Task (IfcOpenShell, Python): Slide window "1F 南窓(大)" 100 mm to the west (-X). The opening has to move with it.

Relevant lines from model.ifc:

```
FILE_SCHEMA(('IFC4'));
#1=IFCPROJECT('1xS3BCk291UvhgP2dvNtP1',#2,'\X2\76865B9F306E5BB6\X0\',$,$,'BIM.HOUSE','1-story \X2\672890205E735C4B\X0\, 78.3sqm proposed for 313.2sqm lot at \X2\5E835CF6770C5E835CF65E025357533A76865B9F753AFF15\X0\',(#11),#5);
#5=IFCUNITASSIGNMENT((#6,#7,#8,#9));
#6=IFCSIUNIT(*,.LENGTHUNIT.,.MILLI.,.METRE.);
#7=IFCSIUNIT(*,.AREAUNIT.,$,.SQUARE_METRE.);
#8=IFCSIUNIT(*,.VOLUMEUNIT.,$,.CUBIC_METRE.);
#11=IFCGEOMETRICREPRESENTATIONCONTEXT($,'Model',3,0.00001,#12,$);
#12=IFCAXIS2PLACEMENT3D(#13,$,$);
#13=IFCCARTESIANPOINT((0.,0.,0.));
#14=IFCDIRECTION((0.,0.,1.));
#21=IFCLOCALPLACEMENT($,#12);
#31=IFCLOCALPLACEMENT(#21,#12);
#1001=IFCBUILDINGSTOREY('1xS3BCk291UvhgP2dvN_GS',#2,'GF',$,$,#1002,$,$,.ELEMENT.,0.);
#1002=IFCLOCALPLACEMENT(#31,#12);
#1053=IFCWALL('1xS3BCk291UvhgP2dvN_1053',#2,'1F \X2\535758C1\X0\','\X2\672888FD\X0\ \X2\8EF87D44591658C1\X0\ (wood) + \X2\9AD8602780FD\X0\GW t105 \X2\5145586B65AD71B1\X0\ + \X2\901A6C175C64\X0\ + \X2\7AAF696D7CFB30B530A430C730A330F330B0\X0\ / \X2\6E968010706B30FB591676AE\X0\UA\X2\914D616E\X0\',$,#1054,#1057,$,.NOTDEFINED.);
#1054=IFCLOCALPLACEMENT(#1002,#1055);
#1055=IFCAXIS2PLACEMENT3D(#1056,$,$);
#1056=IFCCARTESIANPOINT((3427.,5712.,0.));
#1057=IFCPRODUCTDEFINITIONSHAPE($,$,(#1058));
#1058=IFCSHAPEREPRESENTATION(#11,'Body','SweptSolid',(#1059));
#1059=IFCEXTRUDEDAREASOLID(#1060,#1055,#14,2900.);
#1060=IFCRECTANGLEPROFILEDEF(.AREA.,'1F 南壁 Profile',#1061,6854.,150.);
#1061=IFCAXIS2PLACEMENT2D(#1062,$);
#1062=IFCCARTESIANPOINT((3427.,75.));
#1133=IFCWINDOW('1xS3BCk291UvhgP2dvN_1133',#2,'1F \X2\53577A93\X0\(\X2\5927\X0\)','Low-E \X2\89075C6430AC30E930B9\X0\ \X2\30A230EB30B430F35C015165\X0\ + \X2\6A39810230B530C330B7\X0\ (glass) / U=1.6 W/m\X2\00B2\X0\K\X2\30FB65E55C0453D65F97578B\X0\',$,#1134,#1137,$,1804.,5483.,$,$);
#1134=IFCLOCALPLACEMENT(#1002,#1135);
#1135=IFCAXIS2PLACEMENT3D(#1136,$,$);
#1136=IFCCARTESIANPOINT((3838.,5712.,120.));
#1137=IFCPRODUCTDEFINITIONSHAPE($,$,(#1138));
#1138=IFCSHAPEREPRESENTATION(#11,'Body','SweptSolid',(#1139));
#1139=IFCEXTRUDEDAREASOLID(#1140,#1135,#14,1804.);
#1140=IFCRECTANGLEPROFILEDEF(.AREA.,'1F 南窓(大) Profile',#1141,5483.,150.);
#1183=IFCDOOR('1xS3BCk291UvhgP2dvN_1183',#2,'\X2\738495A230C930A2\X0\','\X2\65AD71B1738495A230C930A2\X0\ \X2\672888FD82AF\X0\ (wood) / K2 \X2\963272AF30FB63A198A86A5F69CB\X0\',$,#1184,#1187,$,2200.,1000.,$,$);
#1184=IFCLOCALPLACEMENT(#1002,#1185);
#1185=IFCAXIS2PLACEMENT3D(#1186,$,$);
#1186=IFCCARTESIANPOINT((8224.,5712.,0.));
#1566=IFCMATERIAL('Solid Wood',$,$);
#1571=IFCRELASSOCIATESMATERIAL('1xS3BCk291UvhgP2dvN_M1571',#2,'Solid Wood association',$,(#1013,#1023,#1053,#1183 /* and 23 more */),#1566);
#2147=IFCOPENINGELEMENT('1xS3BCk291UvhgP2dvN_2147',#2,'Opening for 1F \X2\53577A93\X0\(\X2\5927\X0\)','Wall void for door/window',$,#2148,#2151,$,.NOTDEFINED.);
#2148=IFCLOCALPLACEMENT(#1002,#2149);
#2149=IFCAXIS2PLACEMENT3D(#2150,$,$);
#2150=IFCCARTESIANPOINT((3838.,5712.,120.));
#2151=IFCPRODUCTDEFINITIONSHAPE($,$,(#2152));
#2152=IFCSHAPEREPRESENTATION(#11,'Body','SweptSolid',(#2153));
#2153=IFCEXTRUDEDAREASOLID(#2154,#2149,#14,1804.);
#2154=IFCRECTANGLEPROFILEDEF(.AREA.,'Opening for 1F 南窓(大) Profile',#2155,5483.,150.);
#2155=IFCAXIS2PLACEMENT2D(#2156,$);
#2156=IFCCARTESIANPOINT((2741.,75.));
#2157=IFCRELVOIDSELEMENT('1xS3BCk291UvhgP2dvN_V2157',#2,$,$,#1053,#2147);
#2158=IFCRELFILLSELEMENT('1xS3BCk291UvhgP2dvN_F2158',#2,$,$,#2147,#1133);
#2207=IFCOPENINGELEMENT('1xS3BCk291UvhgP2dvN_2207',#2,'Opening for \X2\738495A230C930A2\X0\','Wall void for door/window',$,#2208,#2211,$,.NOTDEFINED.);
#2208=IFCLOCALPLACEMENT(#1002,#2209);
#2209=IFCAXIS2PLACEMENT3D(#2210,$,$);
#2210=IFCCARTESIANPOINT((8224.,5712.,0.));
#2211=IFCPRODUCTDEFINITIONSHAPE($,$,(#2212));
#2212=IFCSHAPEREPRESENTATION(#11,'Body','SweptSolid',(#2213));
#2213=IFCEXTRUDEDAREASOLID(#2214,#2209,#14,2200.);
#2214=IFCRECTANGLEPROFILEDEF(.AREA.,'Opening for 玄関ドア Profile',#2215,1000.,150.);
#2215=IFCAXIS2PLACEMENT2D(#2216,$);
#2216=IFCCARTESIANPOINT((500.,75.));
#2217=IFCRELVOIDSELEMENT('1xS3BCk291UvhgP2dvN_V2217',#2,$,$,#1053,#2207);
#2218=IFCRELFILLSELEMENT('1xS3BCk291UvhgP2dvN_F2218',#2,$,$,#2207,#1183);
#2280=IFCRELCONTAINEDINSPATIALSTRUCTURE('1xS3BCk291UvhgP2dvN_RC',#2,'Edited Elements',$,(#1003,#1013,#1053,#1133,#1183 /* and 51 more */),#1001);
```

```python
import ifcopenshell
import ifcopenshell.api.geometry
import ifcopenshell.util.placement

model = ifcopenshell.open("model.ifc")

window = model.by_guid("1xS3BCk291UvhgP2dvN_1133")
opening = window.FillsVoids[0].RelatingOpeningElement
wall = opening.VoidsElements[0].RelatingBuildingElement

wall_matrix = ifcopenshell.util.placement.get_local_placement(wall.ObjectPlacement)
shift = wall_matrix[:3, 0] * -100.0
before = ifcopenshell.util.placement.get_local_placement(window.ObjectPlacement)[:3, 3].copy()

# The window is not placed relative to its opening, so move both.
for product in (opening, window):
    matrix = ifcopenshell.util.placement.get_local_placement(product.ObjectPlacement)
    matrix[:3, 3] += shift
    ifcopenshell.api.geometry.edit_object_placement(model, product=product, matrix=matrix, is_si=False)

after = ifcopenshell.util.placement.get_local_placement(window.ObjectPlacement)[:3, 3]
print("window moved by", (after - before).round(3) + 0.0)

model.write("model_rev.ifc")
```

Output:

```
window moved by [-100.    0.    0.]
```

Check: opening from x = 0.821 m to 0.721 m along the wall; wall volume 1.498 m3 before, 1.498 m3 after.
